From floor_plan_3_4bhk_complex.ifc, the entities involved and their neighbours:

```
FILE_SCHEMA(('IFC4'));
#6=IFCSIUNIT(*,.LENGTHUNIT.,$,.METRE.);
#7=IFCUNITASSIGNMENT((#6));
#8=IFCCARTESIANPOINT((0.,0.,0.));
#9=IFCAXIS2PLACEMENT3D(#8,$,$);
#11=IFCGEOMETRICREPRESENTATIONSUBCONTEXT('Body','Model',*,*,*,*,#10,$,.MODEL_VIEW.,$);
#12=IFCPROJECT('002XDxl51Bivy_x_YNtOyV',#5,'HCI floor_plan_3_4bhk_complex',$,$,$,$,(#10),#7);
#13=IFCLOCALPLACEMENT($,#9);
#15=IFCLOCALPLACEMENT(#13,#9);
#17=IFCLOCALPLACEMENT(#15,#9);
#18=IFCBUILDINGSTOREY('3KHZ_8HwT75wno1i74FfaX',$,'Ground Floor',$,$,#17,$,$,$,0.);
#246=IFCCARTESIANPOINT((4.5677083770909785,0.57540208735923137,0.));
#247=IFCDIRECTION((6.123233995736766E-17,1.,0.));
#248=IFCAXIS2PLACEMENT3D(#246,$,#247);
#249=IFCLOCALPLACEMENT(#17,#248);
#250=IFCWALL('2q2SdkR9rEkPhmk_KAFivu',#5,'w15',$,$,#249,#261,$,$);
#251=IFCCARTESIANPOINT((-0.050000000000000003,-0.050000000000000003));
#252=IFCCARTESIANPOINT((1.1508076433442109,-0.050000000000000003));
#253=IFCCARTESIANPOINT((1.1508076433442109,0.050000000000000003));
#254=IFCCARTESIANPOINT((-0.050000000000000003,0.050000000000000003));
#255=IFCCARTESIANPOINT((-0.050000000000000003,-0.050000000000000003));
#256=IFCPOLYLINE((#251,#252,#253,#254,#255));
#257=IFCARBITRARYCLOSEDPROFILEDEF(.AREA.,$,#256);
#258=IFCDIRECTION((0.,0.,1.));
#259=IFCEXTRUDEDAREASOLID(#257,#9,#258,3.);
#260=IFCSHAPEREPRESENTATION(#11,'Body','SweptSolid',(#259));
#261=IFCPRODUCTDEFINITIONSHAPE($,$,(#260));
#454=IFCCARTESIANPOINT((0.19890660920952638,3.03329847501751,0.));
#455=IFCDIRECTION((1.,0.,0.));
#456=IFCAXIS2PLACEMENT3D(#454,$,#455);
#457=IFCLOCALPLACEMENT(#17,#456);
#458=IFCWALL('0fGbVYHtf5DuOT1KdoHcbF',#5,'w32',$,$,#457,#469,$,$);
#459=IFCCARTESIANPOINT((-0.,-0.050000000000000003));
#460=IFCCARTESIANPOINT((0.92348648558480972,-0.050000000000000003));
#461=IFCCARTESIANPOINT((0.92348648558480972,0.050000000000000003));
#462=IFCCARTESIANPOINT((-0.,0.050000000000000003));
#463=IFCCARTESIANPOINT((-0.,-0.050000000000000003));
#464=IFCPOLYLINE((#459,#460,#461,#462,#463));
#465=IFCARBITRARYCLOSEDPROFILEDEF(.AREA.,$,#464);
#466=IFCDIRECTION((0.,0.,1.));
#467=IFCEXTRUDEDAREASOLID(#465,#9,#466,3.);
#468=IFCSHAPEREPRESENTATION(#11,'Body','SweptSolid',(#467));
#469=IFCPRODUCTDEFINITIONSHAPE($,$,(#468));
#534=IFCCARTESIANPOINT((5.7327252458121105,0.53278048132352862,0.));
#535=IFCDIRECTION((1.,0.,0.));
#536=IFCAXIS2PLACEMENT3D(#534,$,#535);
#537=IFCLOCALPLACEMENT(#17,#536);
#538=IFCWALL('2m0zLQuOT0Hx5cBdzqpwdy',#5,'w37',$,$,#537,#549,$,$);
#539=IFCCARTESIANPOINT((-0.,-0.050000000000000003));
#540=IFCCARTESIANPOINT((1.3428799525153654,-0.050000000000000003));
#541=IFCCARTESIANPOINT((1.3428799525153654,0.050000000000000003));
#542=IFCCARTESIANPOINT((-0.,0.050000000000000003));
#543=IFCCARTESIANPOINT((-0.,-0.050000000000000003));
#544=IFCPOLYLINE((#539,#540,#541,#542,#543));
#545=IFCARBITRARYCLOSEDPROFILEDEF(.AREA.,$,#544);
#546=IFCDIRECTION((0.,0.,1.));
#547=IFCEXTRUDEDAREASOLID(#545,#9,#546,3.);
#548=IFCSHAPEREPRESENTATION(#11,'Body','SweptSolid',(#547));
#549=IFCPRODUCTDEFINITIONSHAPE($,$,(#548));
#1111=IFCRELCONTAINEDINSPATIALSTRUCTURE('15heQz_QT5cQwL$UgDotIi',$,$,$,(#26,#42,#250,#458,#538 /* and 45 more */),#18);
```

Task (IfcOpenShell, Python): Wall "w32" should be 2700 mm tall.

```python
import ifcopenshell
import ifcopenshell.geom
import ifcopenshell.util.representation
import ifcopenshell.util.shape

model = ifcopenshell.open("floor_plan_3_4bhk_complex.ifc")
settings = ifcopenshell.geom.settings()


def volume(element):
    """Net volume in cubic metres, openings subtracted."""
    shape = ifcopenshell.geom.create_shape(settings, element)
    return ifcopenshell.util.shape.get_volume(shape.geometry)


wall = model.by_guid("0fGbVYHtf5DuOT1KdoHcbF")
before = volume(wall)

body = ifcopenshell.util.representation.get_representation(wall, "Model", "Body")
solid = body.Items[0]
old_height = solid.Depth
solid.Depth = 2.7
after = volume(wall)

print(f"height {old_height:g} -> {solid.Depth:g}, volume {before:.3f} -> {after:.3f} m3")

model.write("floor_plan_3_4bhk_complex_rev.ifc")
```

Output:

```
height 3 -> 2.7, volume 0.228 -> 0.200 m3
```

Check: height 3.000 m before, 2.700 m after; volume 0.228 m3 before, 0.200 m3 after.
